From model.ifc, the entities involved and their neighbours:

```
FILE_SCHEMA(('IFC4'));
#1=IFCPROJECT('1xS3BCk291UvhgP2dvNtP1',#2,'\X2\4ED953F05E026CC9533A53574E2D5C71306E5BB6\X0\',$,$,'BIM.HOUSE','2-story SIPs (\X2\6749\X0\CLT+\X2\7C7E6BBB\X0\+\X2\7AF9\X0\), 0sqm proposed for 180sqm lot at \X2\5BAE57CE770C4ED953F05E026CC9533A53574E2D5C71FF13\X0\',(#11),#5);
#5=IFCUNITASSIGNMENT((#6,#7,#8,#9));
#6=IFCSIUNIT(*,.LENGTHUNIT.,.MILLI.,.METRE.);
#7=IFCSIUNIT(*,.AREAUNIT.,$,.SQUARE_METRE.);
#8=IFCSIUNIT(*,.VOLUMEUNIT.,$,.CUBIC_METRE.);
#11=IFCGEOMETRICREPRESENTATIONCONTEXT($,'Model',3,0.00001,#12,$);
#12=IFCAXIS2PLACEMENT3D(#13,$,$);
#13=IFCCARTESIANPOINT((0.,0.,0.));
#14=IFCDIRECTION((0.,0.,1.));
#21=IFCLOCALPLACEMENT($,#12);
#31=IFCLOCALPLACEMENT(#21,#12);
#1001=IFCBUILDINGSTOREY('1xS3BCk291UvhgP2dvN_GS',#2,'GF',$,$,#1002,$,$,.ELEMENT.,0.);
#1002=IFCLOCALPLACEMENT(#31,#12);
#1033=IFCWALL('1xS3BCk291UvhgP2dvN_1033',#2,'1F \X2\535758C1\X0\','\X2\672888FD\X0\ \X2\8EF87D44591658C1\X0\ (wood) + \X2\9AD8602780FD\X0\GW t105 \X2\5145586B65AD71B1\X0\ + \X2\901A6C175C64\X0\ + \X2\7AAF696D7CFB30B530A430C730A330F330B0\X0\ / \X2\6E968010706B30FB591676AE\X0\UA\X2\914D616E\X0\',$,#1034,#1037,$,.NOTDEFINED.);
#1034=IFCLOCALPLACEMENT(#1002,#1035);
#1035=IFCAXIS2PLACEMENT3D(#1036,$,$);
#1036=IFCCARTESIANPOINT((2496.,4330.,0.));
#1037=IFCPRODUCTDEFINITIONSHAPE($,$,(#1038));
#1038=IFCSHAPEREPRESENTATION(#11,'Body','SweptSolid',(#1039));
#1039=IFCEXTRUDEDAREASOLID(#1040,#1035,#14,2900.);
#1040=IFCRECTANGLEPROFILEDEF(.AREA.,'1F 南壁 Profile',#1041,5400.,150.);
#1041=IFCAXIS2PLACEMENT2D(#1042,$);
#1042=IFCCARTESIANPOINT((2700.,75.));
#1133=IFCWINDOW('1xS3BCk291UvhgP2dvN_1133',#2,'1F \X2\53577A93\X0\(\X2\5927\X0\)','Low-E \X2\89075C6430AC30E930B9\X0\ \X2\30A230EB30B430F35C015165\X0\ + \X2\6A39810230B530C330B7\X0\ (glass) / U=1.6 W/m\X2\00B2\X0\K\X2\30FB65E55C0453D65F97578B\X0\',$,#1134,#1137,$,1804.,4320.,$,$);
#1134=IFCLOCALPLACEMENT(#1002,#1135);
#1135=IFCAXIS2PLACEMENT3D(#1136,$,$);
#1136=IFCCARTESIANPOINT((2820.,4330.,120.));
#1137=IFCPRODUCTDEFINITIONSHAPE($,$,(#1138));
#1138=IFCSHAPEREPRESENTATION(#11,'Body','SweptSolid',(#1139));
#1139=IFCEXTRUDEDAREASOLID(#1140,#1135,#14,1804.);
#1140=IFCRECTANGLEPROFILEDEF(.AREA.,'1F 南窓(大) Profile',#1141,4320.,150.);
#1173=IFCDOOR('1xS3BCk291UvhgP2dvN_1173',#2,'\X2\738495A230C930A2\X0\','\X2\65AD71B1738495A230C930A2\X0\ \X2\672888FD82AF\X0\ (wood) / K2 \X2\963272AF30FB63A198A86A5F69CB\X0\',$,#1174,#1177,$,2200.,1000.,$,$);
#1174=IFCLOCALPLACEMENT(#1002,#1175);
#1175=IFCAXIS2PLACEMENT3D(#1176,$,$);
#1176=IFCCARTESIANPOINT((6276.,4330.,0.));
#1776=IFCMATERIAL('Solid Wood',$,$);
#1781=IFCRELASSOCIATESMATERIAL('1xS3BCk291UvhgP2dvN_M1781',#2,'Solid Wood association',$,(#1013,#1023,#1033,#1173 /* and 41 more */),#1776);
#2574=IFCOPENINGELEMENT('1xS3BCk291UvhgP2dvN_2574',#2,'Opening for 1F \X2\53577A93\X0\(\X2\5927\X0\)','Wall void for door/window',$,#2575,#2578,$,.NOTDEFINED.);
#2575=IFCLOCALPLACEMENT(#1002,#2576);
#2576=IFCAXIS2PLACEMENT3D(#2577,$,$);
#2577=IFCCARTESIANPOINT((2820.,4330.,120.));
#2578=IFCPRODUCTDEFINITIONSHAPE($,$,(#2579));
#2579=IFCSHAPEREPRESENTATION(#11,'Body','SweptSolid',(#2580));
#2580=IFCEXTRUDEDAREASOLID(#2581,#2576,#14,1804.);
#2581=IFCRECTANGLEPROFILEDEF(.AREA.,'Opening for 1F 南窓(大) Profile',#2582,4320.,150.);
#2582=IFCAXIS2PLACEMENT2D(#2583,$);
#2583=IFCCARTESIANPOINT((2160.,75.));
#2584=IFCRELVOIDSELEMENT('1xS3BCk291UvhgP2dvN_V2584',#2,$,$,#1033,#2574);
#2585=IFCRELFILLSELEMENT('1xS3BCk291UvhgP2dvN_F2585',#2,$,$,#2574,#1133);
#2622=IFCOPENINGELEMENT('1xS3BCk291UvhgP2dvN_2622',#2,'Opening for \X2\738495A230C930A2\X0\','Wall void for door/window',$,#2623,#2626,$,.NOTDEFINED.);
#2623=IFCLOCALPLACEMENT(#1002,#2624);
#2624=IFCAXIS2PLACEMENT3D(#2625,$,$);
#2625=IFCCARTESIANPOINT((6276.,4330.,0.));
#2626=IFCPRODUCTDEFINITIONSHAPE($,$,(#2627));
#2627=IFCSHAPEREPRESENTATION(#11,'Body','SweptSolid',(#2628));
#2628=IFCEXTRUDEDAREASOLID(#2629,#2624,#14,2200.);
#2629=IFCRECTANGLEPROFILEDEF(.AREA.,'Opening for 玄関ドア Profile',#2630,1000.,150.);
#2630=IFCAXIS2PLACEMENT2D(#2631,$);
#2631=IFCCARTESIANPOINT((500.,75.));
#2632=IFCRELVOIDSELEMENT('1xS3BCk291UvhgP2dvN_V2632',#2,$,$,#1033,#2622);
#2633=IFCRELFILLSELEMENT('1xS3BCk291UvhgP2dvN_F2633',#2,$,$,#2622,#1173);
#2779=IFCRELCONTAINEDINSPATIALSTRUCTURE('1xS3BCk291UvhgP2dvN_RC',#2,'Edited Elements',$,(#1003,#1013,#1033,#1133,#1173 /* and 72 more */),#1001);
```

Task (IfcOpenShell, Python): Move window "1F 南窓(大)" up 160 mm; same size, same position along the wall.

```python
import numpy as np
import ifcopenshell
import ifcopenshell.api.geometry
import ifcopenshell.util.placement
import ifcopenshell.util.unit

model = ifcopenshell.open("model.ifc")
unit_scale = ifcopenshell.util.unit.calculate_unit_scale(model)

window = model.by_guid("1xS3BCk291UvhgP2dvN_1133")
opening = window.FillsVoids[0].RelatingOpeningElement
dz = 0.16 / unit_scale

shift = np.array([0.0, 0.0, dz])
# The window is not placed relative to its opening, so move both.
for product in (opening, window):
    matrix = ifcopenshell.util.placement.get_local_placement(product.ObjectPlacement)
    matrix[:3, 3] += shift
    ifcopenshell.api.geometry.edit_object_placement(model, product=product, matrix=matrix, is_si=False)

print(f"moved by {dz * unit_scale:+.3f} m")

model.write("model_edited.ifc")
```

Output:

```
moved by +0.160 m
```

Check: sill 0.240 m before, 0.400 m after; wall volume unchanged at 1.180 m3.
